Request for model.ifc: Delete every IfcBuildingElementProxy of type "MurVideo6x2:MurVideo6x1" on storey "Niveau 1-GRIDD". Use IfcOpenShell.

First a look at what the model holds.

```python
import ifcopenshell
import ifcopenshell.util.element

model = ifcopenshell.open("model.ifc")
print(model.schema)
storey = next(s for s in model.by_type("IfcBuildingStorey") if s.Name == "Niveau 1-GRIDD")
proxies = [e for e in ifcopenshell.util.element.get_decomposition(storey) if e.is_a("IfcBuildingElementProxy")]
seen = {}
for e in proxies:
    element_type = ifcopenshell.util.element.get_type(e)
    name = element_type.Name if element_type not in (None, e) else None
    seen[name] = seen.get(name, 0) + 1
for name, count in sorted(seen.items(), key=str):
    print(count, "x", name)
```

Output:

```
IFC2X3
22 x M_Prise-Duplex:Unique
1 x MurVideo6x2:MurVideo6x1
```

```python
import ifcopenshell
import ifcopenshell.api.root
import ifcopenshell.util.element

model = ifcopenshell.open("model.ifc")

storey = next(s for s in model.by_type("IfcBuildingStorey") if s.Name == "Niveau 1-GRIDD")
proxies = [e for e in ifcopenshell.util.element.get_decomposition(storey) if e.is_a("IfcBuildingElementProxy")]
targets = [e for e in proxies if (t := ifcopenshell.util.element.get_type(e)) not in (None, e) and t.Name == "MurVideo6x2:MurVideo6x1"]

for e in targets:
    ifcopenshell.api.root.remove_product(model, product=e)
print(len(targets), "removed")

model.write("model_edited.ifc")
```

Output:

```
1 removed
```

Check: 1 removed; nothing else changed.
